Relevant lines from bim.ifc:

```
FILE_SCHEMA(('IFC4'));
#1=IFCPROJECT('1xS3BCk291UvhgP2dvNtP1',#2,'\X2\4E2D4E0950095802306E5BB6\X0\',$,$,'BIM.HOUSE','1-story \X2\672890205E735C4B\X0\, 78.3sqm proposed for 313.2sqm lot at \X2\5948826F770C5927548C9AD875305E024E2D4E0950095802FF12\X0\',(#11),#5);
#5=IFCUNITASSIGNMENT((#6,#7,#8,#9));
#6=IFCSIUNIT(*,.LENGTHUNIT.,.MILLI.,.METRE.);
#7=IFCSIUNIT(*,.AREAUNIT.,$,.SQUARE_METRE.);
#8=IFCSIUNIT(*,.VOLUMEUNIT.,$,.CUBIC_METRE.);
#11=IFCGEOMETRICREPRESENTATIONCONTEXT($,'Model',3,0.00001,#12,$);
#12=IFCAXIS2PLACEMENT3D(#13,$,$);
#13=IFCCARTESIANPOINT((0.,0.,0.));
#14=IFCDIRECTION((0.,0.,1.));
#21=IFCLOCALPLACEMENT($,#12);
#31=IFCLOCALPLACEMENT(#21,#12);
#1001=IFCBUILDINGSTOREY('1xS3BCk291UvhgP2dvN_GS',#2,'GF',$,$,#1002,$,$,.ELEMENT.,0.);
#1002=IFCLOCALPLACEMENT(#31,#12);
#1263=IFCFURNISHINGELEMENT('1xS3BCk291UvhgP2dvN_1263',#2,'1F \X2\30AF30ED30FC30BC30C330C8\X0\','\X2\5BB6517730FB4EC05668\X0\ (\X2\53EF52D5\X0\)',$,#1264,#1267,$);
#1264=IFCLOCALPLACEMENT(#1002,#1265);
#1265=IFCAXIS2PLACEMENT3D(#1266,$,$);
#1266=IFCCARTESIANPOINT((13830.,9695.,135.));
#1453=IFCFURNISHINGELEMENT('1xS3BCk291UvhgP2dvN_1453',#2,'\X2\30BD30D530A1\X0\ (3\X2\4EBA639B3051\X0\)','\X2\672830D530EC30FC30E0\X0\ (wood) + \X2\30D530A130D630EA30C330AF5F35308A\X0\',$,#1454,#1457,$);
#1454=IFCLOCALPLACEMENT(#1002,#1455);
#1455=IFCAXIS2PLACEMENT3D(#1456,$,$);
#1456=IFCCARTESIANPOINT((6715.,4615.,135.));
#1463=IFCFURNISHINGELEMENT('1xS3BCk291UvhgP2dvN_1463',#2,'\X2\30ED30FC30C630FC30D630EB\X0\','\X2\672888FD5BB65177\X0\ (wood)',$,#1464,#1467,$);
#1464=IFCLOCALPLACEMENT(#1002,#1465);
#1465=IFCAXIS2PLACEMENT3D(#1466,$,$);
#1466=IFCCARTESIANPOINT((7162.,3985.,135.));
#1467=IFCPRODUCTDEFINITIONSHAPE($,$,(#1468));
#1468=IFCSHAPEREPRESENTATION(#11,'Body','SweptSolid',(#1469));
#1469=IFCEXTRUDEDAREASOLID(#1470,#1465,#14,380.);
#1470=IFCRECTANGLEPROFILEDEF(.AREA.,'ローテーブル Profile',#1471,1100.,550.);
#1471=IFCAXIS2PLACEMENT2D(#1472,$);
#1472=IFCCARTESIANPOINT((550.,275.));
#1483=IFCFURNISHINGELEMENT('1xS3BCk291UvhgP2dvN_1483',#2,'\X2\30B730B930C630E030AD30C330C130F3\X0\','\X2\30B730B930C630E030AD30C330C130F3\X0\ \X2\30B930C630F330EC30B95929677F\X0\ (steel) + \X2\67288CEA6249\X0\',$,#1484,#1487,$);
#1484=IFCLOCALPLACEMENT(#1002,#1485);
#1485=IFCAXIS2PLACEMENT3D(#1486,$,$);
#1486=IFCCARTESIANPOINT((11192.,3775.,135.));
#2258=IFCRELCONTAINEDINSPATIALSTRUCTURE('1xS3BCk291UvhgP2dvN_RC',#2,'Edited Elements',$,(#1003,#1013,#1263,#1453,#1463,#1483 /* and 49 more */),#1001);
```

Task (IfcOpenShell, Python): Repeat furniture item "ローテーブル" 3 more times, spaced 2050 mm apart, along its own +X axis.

```python
import ifcopenshell
import ifcopenshell.api.geometry
import ifcopenshell.api.root
import ifcopenshell.util.element
import ifcopenshell.util.placement

model = ifcopenshell.open("bim.ifc")


def reuse_history(source, copy):
    """copy_class also copies each property set's owner history, people and application; keep the originals."""
    for rel in copy.IsDefinedBy:
        if rel.is_a("IfcRelDefinesByProperties") and (history := rel.RelatingPropertyDefinition.OwnerHistory):
            rel.RelatingPropertyDefinition.OwnerHistory = source.OwnerHistory
            ifcopenshell.util.element.remove_deep2(model, history)


source = model.by_guid("1xS3BCk291UvhgP2dvN_1463")
base = ifcopenshell.util.placement.get_local_placement(source.ObjectPlacement)
step = base[:3, 0] * 2050.0

for i in range(1, 4):
    copy = ifcopenshell.api.root.copy_class(model, product=source)
    copy.Representation = ifcopenshell.util.element.copy_deep(
        model, source.Representation, exclude=["IfcGeometricRepresentationContext", "IfcRepresentationMap"]
    )
    reuse_history(source, copy)
    matrix = base.copy()
    matrix[:3, 3] += i * step
    print("added at", matrix[:3, 3].round(3) + 0.0)
    ifcopenshell.api.geometry.edit_object_placement(model, product=copy, matrix=matrix, is_si=False)

model.write("bim_edited.ifc")
```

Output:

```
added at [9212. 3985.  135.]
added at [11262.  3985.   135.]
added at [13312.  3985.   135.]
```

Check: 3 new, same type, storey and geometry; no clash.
